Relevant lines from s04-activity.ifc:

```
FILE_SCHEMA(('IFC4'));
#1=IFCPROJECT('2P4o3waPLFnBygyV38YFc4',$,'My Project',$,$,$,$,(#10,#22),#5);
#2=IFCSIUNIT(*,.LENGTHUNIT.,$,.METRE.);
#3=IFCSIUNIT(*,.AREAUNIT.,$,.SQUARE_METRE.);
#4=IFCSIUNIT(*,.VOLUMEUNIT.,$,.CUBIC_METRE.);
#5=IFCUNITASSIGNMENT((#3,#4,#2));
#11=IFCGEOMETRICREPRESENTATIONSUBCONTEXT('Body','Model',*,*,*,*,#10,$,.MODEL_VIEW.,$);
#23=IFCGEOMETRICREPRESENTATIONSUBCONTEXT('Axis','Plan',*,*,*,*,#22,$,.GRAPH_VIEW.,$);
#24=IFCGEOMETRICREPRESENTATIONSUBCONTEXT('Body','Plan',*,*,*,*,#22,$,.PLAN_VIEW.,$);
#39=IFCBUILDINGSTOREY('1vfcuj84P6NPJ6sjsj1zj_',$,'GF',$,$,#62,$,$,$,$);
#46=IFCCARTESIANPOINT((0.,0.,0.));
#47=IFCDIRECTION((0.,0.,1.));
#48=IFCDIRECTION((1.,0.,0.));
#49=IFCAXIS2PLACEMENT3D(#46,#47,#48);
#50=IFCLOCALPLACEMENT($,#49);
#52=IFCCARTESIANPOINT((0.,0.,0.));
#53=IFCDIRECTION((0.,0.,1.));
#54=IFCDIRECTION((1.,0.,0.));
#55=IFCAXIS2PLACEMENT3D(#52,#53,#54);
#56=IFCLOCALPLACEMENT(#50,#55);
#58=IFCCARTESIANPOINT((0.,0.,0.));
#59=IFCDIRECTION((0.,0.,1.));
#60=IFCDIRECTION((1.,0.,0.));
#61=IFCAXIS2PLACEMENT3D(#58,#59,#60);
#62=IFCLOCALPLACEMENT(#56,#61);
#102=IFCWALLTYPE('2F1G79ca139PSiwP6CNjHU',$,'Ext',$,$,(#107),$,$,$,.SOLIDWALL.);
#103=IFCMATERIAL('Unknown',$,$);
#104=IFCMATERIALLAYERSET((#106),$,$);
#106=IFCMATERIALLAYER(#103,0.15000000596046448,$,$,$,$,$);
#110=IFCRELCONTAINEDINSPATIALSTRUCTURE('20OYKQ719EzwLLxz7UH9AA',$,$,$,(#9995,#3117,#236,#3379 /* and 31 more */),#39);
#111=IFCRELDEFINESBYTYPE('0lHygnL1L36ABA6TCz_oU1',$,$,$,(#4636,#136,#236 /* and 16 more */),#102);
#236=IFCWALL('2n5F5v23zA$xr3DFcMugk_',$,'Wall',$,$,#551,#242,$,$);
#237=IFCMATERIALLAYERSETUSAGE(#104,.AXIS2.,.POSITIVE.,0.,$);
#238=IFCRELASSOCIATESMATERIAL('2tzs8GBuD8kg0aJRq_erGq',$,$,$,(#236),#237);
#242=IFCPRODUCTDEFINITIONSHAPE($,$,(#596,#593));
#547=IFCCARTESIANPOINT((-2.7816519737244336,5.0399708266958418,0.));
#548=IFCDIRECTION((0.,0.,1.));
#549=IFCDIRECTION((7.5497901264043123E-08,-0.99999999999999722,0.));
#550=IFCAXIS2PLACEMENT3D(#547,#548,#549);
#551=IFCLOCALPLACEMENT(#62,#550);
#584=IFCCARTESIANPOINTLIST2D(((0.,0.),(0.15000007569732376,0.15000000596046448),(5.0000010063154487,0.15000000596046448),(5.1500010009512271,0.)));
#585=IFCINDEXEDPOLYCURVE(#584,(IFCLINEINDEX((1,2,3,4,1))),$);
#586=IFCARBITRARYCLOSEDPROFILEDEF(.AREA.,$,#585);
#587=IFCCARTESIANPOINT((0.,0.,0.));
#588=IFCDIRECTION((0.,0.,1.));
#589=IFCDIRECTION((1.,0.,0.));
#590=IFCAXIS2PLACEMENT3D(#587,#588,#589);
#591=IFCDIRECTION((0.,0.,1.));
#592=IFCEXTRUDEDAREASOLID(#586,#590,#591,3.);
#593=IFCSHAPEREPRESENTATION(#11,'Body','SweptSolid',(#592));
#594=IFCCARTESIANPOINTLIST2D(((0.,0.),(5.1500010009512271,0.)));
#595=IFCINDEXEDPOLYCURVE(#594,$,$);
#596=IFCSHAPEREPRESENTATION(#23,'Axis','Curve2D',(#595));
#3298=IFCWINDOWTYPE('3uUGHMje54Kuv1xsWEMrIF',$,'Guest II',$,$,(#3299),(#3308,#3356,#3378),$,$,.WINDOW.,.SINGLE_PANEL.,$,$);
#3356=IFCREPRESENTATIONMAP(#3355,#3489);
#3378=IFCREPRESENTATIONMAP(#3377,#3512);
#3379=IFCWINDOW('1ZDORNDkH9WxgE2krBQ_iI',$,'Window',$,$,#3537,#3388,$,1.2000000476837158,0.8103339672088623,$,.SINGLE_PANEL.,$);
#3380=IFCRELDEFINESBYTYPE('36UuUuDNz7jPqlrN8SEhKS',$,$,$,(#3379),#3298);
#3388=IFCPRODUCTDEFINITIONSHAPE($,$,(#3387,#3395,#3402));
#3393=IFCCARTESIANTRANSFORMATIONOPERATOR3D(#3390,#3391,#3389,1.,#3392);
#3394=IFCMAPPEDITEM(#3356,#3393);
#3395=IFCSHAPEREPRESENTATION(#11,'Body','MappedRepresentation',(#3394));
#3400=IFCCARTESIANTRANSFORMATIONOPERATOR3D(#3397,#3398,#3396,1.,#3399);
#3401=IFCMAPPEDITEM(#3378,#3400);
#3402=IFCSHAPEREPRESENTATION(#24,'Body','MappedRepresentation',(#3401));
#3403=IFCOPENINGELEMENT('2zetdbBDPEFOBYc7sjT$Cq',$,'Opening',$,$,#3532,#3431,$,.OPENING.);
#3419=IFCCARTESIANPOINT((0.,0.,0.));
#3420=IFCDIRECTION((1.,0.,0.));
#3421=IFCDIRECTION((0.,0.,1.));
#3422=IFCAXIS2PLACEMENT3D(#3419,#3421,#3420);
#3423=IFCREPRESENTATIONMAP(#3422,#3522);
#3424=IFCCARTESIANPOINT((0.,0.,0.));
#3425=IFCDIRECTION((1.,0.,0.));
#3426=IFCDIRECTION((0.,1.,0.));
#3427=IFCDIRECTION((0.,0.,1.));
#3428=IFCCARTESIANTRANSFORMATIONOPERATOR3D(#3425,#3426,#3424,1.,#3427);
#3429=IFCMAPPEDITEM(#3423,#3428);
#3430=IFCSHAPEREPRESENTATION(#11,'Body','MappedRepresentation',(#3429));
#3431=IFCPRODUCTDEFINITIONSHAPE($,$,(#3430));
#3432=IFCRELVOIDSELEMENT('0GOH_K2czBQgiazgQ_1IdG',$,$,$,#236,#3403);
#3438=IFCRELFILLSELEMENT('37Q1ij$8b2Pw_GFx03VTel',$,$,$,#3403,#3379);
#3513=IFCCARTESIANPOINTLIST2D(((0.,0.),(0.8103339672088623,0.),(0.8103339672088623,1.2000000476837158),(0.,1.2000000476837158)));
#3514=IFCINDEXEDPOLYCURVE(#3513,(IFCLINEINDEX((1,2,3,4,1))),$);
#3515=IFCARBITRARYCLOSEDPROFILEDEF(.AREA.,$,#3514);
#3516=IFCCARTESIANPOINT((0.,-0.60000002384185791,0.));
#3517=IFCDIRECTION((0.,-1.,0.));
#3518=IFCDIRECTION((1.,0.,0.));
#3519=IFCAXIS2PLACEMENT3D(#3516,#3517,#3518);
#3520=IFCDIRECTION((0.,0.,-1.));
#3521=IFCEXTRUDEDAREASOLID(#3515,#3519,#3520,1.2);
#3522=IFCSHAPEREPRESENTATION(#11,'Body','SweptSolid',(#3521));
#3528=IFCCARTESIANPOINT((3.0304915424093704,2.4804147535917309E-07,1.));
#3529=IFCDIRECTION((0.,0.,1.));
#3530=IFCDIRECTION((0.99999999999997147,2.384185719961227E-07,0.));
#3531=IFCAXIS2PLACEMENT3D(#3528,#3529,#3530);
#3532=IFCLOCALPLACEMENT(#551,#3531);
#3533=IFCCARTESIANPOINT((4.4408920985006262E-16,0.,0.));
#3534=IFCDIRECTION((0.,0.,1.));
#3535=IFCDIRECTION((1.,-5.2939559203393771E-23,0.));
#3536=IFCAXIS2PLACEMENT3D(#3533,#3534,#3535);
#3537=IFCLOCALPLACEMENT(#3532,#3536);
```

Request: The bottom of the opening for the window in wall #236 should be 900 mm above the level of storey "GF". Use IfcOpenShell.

```python
import numpy as np
import ifcopenshell
import ifcopenshell.api.geometry
import ifcopenshell.geom
import ifcopenshell.util.element
import ifcopenshell.util.placement
import ifcopenshell.util.shape
import ifcopenshell.util.unit

model = ifcopenshell.open("s04-activity.ifc")
unit_scale = ifcopenshell.util.unit.calculate_unit_scale(model)

window = model.by_guid("1ZDORNDkH9WxgE2krBQ_iI")
opening = window.FillsVoids[0].RelatingOpeningElement
storey = ifcopenshell.util.element.get_container(window, ifc_class="IfcBuildingStorey")
level = ifcopenshell.util.placement.get_local_placement(storey.ObjectPlacement)[2, 3]

# The opening's origin need not be at the sill, so measure its lowest point.
shape = ifcopenshell.geom.create_shape(ifcopenshell.geom.settings(), opening)
bottom = ifcopenshell.util.shape.get_shape_bottom_elevation(shape, shape.geometry) / unit_scale
dz = level + 0.9 - bottom

shift = np.array([0.0, 0.0, dz])
# The window is placed relative to its opening, so it follows when the opening moves.
matrix = ifcopenshell.util.placement.get_local_placement(opening.ObjectPlacement)
matrix[:3, 3] += shift
ifcopenshell.api.geometry.edit_object_placement(
    model, product=opening, matrix=matrix, is_si=False, should_transform_children=True
)

print(f"moved by {dz * unit_scale:+.3f} m")

model.write("s04-activity_updated.ifc")
```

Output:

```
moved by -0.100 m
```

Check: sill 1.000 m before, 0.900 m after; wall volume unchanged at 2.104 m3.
